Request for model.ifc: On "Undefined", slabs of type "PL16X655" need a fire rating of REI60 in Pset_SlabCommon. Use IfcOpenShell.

First a look at what the model holds.

```python
import ifcopenshell
import ifcopenshell.util.element

model = ifcopenshell.open("model.ifc")
print(model.schema)
storey = next(s for s in model.by_type("IfcBuildingStorey") if s.Name == "Undefined")
slabs = [e for e in ifcopenshell.util.element.get_decomposition(storey) if e.is_a("IfcSlab")]
seen = {}
for e in slabs:
    element_type = ifcopenshell.util.element.get_type(e)
    key = (element_type.Name if element_type != e and element_type else None, ifcopenshell.util.element.get_pset(e, "Pset_SlabCommon", "FireRating"))
    seen[key] = seen.get(key, 0) + 1
for (name, value), count in sorted(seen.items(), key=str):
    print(count, "x", name, "|", value)
```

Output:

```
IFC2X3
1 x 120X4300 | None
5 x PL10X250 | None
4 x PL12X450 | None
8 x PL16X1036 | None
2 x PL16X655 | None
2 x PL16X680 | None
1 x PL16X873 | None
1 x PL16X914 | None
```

```python
import ifcopenshell
import ifcopenshell.api.pset
import ifcopenshell.util.element

model = ifcopenshell.open("model.ifc")

storey = next(s for s in model.by_type("IfcBuildingStorey") if s.Name == "Undefined")
slabs = [e for e in ifcopenshell.util.element.get_decomposition(storey) if e.is_a("IfcSlab")]

count = 0
for e in slabs:
    element_type = ifcopenshell.util.element.get_type(e)
    if element_type in (None, e) or element_type.Name != "PL16X655":
        continue
    # add_pset returns the element's existing set when there is one.
    pset = ifcopenshell.api.pset.add_pset(model, product=e, name="Pset_SlabCommon")
    ifcopenshell.api.pset.edit_pset(model, pset=pset, properties={"FireRating": "REI60"})
    count += 1

print(count, "slabs updated")

model.write("model_v2.ifc")
```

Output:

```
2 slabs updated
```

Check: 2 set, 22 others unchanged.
